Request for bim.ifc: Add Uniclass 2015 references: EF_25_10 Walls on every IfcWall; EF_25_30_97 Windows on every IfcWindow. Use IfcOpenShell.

First a look at what the model holds.

```python
import ifcopenshell

model = ifcopenshell.open("bim.ifc")
print(model.schema)
print("classifications:", [c.Name for c in model.by_type("IfcClassification")])
for ifc_class in ("IfcDoor", "IfcRoof", "IfcStair", "IfcWall", "IfcWindow"):
    print(ifc_class, len(model.by_type(ifc_class)))
```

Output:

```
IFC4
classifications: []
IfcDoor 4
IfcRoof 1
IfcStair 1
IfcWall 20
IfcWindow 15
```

```python
import ifcopenshell
import ifcopenshell.api.classification

model = ifcopenshell.open("bim.ifc")

system = ifcopenshell.api.classification.add_classification(model, classification="Uniclass 2015")

codes = {
    "IfcWall": ("EF_25_10", "Walls"),
    "IfcWindow": ("EF_25_30_97", "Windows"),
}
for ifc_class, (code, name) in codes.items():
    products = model.by_type(ifc_class)
    ifcopenshell.api.classification.add_reference(
        model, products=products, classification=system, identification=code, name=name
    )
    print(code, len(products))

model.write("bim_v2.ifc")
```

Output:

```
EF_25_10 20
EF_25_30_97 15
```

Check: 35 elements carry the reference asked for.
